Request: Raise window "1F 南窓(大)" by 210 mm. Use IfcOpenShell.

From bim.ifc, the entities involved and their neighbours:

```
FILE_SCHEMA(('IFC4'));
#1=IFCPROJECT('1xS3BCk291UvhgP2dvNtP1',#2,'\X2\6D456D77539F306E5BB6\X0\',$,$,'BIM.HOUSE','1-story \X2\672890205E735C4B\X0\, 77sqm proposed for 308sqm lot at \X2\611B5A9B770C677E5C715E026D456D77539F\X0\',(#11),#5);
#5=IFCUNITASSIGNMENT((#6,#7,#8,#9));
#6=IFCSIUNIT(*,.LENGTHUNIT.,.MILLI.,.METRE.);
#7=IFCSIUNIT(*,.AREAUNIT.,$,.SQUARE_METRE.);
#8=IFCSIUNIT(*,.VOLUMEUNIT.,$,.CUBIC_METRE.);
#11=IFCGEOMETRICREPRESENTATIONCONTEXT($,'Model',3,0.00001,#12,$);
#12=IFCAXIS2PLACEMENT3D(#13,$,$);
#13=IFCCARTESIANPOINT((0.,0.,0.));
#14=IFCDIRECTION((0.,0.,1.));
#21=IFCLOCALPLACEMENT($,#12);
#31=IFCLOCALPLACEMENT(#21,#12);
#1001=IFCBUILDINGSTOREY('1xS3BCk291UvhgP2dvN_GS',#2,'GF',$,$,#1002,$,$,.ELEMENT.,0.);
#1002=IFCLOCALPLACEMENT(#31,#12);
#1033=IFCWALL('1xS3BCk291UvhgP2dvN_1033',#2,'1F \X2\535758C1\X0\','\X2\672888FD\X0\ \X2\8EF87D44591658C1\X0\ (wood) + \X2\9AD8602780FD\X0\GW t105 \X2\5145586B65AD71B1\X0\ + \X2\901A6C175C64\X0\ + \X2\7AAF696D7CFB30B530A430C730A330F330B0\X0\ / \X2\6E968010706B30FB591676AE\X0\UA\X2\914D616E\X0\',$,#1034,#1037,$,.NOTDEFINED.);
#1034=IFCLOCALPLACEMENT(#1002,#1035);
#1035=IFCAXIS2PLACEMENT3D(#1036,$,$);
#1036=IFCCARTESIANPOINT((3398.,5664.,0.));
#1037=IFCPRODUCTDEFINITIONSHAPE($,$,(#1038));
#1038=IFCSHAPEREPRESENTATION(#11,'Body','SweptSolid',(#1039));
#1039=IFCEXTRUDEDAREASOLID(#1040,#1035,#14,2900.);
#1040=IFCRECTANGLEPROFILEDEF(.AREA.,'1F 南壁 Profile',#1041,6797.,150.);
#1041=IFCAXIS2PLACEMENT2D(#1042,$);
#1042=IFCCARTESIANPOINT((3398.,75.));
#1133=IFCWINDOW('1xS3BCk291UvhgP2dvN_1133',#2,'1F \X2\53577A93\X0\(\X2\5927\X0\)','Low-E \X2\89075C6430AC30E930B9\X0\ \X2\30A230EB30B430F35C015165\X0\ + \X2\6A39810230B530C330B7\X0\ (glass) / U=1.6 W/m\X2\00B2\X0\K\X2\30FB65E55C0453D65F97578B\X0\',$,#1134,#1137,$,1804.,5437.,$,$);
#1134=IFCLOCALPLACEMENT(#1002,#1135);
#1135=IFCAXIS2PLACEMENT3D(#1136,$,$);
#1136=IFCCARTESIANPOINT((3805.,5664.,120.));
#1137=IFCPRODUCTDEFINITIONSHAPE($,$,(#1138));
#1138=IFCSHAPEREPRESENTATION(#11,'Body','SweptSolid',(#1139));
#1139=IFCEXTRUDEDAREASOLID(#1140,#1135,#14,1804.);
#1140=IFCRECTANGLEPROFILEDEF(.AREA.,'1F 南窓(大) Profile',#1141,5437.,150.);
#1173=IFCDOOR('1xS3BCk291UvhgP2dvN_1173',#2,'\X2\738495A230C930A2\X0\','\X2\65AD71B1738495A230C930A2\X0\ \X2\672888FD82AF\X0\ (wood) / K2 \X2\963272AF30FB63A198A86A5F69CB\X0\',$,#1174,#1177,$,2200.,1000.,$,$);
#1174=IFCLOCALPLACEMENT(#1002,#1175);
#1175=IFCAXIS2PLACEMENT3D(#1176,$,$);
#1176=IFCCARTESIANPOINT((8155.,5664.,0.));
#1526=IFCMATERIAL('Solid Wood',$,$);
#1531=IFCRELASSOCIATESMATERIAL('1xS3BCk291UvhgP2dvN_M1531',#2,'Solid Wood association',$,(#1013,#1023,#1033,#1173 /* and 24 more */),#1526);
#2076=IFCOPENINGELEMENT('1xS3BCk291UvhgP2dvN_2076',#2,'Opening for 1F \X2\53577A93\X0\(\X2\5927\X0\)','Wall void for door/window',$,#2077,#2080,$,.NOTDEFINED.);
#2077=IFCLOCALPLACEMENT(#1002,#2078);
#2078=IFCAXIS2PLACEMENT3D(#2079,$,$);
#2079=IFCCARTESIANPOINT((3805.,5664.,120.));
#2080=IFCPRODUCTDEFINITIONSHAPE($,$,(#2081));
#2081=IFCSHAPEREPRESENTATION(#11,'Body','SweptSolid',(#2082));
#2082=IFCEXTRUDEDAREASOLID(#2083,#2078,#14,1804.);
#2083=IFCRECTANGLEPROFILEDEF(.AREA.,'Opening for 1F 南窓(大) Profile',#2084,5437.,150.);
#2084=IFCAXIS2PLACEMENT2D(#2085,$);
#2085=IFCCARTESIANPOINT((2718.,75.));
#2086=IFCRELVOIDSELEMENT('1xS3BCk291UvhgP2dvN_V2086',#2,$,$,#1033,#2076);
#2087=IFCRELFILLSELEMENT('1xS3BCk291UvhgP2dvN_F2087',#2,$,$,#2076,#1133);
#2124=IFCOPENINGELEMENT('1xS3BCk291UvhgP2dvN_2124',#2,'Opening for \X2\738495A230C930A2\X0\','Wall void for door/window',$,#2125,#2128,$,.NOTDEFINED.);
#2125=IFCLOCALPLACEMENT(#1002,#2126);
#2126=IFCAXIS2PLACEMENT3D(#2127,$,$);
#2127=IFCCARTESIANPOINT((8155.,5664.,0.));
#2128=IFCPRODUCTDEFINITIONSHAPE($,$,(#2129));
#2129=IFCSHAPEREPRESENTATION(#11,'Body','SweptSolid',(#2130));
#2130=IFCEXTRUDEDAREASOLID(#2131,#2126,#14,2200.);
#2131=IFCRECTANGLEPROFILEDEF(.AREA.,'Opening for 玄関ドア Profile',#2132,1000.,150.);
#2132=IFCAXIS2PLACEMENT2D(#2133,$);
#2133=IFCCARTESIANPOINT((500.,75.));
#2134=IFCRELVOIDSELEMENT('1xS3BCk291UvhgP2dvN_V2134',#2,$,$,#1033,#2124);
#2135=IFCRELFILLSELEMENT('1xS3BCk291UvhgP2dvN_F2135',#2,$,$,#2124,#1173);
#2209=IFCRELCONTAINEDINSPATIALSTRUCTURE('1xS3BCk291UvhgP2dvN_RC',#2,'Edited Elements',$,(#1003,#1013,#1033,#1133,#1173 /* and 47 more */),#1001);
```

```python
import numpy as np
import ifcopenshell
import ifcopenshell.api.geometry
import ifcopenshell.util.placement
import ifcopenshell.util.unit

model = ifcopenshell.open("bim.ifc")
unit_scale = ifcopenshell.util.unit.calculate_unit_scale(model)

window = model.by_guid("1xS3BCk291UvhgP2dvN_1133")
opening = window.FillsVoids[0].RelatingOpeningElement
dz = 0.21 / unit_scale

shift = np.array([0.0, 0.0, dz])
# The window is not placed relative to its opening, so move both.
for product in (opening, window):
    matrix = ifcopenshell.util.placement.get_local_placement(product.ObjectPlacement)
    matrix[:3, 3] += shift
    ifcopenshell.api.geometry.edit_object_placement(model, product=product, matrix=matrix, is_si=False)

print(f"moved by {dz * unit_scale:+.3f} m")

model.write("bim_rev.ifc")
```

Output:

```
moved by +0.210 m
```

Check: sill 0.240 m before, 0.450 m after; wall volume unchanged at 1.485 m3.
